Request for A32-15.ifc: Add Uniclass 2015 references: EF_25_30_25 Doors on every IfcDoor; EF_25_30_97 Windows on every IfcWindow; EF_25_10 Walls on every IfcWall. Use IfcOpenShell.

First a look at what the model holds.

```python
import ifcopenshell

model = ifcopenshell.open("A32-15.ifc")
print(model.schema)
print("classifications:", [c.Name for c in model.by_type("IfcClassification")])
for ifc_class in ("IfcDoor", "IfcRoof", "IfcStair", "IfcWall", "IfcWindow"):
    print(ifc_class, len(model.by_type(ifc_class)))
```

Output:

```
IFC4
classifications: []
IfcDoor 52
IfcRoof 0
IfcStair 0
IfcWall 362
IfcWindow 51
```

```python
import ifcopenshell
import ifcopenshell.api.classification

model = ifcopenshell.open("A32-15.ifc")

system = ifcopenshell.api.classification.add_classification(model, classification="Uniclass 2015")

codes = {
    "IfcDoor": ("EF_25_30_25", "Doors"),
    "IfcWindow": ("EF_25_30_97", "Windows"),
    "IfcWall": ("EF_25_10", "Walls"),
}
for ifc_class, (code, name) in codes.items():
    products = model.by_type(ifc_class)
    ifcopenshell.api.classification.add_reference(
        model, products=products, classification=system, identification=code, name=name
    )
    print(code, len(products))

model.write("A32-15_updated.ifc")
```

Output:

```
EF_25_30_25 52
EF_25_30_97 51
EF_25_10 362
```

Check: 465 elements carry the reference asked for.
